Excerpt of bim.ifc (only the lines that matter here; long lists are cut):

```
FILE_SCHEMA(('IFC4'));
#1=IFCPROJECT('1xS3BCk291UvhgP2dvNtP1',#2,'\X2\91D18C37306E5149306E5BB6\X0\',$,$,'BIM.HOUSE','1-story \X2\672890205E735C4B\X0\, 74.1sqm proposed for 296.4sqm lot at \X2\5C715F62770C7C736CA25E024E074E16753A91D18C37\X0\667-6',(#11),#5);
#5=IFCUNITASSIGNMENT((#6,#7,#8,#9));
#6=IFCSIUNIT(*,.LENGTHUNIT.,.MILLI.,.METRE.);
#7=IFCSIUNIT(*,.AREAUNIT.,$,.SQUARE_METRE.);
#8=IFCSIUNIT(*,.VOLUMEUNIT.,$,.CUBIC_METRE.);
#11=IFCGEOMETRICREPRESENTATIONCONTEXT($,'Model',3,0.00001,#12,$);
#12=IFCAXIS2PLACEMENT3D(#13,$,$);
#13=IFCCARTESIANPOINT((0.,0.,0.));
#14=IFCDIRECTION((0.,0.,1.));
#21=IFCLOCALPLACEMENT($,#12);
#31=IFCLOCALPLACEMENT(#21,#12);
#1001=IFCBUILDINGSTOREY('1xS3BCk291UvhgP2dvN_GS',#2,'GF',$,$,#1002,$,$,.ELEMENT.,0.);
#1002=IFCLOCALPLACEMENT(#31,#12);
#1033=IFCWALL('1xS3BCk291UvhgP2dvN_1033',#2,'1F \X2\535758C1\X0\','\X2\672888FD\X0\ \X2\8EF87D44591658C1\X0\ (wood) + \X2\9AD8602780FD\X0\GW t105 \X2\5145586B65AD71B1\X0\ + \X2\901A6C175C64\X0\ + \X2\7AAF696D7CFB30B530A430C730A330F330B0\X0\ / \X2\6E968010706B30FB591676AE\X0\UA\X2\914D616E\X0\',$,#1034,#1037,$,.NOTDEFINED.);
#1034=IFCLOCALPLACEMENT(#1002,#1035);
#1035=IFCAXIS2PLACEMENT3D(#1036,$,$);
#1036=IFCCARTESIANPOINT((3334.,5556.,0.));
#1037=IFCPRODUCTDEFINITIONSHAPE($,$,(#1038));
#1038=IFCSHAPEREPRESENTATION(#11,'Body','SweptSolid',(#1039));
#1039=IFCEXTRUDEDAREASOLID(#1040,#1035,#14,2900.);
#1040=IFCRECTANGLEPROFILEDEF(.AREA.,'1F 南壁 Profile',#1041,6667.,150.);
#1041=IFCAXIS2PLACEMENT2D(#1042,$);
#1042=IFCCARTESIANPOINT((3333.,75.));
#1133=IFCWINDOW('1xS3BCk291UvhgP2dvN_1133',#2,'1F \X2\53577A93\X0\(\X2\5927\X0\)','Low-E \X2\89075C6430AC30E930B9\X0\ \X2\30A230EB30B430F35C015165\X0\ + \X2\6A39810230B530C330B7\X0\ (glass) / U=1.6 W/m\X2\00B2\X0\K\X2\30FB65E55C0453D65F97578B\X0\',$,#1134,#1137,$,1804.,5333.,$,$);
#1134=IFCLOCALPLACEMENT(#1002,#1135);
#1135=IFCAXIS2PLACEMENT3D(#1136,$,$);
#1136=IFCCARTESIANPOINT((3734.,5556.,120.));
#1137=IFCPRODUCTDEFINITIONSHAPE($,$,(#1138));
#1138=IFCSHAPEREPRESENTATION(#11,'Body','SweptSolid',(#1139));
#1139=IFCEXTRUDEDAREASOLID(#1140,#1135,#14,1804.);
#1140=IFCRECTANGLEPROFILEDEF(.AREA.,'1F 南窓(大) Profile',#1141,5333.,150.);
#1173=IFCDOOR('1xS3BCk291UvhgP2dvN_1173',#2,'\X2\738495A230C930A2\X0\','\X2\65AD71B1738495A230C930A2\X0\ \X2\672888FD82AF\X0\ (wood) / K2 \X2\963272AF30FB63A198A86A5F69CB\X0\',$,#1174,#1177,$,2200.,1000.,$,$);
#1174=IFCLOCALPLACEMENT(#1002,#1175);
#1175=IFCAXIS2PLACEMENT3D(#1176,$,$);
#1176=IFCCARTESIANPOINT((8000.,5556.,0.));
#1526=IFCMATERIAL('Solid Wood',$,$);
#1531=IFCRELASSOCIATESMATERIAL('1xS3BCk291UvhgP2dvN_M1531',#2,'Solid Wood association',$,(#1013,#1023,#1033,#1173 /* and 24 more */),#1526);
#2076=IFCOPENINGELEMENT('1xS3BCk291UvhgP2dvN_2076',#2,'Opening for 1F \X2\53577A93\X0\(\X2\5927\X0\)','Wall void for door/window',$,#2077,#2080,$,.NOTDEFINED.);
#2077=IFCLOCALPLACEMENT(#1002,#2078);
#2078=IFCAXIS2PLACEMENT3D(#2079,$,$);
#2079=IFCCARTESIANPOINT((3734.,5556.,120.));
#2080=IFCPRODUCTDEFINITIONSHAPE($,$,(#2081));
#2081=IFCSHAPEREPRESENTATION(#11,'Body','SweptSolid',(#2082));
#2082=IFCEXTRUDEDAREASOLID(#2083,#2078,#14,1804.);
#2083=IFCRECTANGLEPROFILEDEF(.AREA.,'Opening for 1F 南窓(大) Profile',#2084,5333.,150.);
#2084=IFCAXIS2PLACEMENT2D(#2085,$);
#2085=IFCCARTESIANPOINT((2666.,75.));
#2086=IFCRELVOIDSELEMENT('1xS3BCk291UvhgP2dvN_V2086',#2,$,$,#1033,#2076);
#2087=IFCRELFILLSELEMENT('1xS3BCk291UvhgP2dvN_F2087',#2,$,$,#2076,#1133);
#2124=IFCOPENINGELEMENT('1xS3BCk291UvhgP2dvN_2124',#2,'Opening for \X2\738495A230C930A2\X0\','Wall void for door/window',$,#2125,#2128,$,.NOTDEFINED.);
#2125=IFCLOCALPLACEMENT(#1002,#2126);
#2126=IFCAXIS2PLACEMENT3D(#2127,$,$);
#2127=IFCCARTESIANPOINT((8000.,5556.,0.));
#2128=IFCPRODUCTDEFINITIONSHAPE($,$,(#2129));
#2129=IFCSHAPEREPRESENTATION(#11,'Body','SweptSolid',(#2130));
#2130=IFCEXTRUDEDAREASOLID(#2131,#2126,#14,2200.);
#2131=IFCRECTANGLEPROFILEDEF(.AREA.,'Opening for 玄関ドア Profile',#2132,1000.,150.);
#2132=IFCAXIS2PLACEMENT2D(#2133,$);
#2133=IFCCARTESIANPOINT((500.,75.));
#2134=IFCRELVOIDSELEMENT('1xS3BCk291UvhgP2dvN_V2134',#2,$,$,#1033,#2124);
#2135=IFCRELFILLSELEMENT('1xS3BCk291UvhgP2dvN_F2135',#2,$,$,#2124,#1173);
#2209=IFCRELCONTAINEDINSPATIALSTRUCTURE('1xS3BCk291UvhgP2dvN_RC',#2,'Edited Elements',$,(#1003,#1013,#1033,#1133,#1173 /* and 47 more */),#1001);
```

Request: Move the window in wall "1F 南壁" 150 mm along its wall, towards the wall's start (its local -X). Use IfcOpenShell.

```python
import ifcopenshell
import ifcopenshell.api.geometry
import ifcopenshell.util.placement
import ifcopenshell.util.unit

model = ifcopenshell.open("bim.ifc")
unit_scale = ifcopenshell.util.unit.calculate_unit_scale(model)

window = model.by_guid("1xS3BCk291UvhgP2dvN_1133")
opening = window.FillsVoids[0].RelatingOpeningElement
wall = opening.VoidsElements[0].RelatingBuildingElement

wall_matrix = ifcopenshell.util.placement.get_local_placement(wall.ObjectPlacement)
shift = wall_matrix[:3, 0] * -0.15 / unit_scale
before = ifcopenshell.util.placement.get_local_placement(window.ObjectPlacement)[:3, 3].copy()

# The window is not placed relative to its opening, so move both.
for product in (opening, window):
    matrix = ifcopenshell.util.placement.get_local_placement(product.ObjectPlacement)
    matrix[:3, 3] += shift
    ifcopenshell.api.geometry.edit_object_placement(model, product=product, matrix=matrix, is_si=False)

after = ifcopenshell.util.placement.get_local_placement(window.ObjectPlacement)[:3, 3]
print("window moved by", (after - before).round(3) + 0.0)

model.write("bim_v2.ifc")
```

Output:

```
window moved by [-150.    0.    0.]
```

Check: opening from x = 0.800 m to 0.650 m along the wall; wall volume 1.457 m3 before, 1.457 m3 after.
